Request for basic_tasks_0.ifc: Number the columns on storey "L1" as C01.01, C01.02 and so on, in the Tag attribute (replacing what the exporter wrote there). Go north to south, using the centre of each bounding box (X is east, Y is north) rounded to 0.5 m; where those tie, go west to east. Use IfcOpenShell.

First a look at what the model holds.

```python
import ifcopenshell
import ifcopenshell.util.element
import ifcopenshell.util.placement

model = ifcopenshell.open("basic_tasks_0.ifc")
print(model.schema)
storey = next(s for s in model.by_type("IfcBuildingStorey") if s.Name == "L1")
columns = [e for e in ifcopenshell.util.element.get_decomposition(storey) if e.is_a("IfcColumn")]
for e in sorted(columns, key=lambda e: e.id()):
    origin = ifcopenshell.util.placement.get_local_placement(e.ObjectPlacement)[:3, 3]
    print(e.id(), e.Tag, e.Name, origin.round(2) + 0.0, sep=" | ")
```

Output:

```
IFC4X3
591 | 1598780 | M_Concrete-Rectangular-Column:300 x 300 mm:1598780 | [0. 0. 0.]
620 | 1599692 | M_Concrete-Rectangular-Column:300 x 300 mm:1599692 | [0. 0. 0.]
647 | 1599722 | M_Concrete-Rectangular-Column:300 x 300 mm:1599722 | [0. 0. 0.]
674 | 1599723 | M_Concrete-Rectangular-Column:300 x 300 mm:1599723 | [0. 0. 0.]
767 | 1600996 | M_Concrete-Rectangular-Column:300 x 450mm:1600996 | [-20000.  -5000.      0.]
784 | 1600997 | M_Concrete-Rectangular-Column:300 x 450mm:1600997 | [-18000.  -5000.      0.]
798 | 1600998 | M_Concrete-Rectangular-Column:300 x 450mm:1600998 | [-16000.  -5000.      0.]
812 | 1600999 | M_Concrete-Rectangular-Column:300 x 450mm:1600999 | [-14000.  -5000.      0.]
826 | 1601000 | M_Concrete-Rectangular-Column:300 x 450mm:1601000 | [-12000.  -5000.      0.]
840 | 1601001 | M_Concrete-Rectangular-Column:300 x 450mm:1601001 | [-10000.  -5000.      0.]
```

```python
import ifcopenshell
import ifcopenshell.geom
import ifcopenshell.util.element
import ifcopenshell.util.shape

model = ifcopenshell.open("basic_tasks_0.ifc")
settings = ifcopenshell.geom.settings()
settings.set("use-world-coords", True)


def centre(element):
    shape = ifcopenshell.geom.create_shape(settings, element)
    return ifcopenshell.util.shape.get_bbox_centroid(shape.geometry)


storey = next(s for s in model.by_type("IfcBuildingStorey") if s.Name == "L1")
columns = [e for e in ifcopenshell.util.element.get_decomposition(storey) if e.is_a("IfcColumn")]

# Insertion points can sit at a corner or the storey origin, so sort by the geometry (in metres).
centres = {e: centre(e) for e in columns}
columns.sort(key=lambda e: (-round(centres[e][1] / 0.5), centres[e][0]))

for i, e in enumerate(columns, start=1):
    number = f"C01.{i:02d}"
    e.Tag = number
    print(e.id(), number)

model.write("basic_tasks_0-out.ifc")
```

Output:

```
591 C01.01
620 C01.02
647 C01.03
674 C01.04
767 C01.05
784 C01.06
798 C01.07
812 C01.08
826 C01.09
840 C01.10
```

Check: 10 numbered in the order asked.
